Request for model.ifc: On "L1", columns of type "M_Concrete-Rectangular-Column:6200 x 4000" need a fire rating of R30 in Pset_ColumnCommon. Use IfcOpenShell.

First a look at what the model holds.

```python
import ifcopenshell
import ifcopenshell.util.element

model = ifcopenshell.open("model.ifc")
print(model.schema)
storey = next(s for s in model.by_type("IfcBuildingStorey") if s.Name == "L1")
columns = [e for e in ifcopenshell.util.element.get_decomposition(storey) if e.is_a("IfcColumn")]
seen = {}
for e in columns:
    element_type = ifcopenshell.util.element.get_type(e)
    key = (element_type.Name if element_type != e and element_type else None, ifcopenshell.util.element.get_pset(e, "Pset_ColumnCommon", "FireRating"))
    seen[key] = seen.get(key, 0) + 1
for (name, value), count in sorted(seen.items(), key=str):
    print(count, "x", name, "|", value)
```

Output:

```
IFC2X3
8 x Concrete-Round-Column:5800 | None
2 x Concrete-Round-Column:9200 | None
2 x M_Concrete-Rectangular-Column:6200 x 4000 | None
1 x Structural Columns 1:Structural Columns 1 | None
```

```python
import ifcopenshell
import ifcopenshell.api.pset
import ifcopenshell.util.element

model = ifcopenshell.open("model.ifc")

storey = next(s for s in model.by_type("IfcBuildingStorey") if s.Name == "L1")
columns = [e for e in ifcopenshell.util.element.get_decomposition(storey) if e.is_a("IfcColumn")]

count = 0
for e in columns:
    element_type = ifcopenshell.util.element.get_type(e)
    if element_type in (None, e) or element_type.Name != "M_Concrete-Rectangular-Column:6200 x 4000":
        continue
    # add_pset returns the element's existing set when there is one.
    pset = ifcopenshell.api.pset.add_pset(model, product=e, name="Pset_ColumnCommon")
    ifcopenshell.api.pset.edit_pset(model, pset=pset, properties={"FireRating": "R30"})
    count += 1

print(count, "columns updated")

model.write("model_rev.ifc")
```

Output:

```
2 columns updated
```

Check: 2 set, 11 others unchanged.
